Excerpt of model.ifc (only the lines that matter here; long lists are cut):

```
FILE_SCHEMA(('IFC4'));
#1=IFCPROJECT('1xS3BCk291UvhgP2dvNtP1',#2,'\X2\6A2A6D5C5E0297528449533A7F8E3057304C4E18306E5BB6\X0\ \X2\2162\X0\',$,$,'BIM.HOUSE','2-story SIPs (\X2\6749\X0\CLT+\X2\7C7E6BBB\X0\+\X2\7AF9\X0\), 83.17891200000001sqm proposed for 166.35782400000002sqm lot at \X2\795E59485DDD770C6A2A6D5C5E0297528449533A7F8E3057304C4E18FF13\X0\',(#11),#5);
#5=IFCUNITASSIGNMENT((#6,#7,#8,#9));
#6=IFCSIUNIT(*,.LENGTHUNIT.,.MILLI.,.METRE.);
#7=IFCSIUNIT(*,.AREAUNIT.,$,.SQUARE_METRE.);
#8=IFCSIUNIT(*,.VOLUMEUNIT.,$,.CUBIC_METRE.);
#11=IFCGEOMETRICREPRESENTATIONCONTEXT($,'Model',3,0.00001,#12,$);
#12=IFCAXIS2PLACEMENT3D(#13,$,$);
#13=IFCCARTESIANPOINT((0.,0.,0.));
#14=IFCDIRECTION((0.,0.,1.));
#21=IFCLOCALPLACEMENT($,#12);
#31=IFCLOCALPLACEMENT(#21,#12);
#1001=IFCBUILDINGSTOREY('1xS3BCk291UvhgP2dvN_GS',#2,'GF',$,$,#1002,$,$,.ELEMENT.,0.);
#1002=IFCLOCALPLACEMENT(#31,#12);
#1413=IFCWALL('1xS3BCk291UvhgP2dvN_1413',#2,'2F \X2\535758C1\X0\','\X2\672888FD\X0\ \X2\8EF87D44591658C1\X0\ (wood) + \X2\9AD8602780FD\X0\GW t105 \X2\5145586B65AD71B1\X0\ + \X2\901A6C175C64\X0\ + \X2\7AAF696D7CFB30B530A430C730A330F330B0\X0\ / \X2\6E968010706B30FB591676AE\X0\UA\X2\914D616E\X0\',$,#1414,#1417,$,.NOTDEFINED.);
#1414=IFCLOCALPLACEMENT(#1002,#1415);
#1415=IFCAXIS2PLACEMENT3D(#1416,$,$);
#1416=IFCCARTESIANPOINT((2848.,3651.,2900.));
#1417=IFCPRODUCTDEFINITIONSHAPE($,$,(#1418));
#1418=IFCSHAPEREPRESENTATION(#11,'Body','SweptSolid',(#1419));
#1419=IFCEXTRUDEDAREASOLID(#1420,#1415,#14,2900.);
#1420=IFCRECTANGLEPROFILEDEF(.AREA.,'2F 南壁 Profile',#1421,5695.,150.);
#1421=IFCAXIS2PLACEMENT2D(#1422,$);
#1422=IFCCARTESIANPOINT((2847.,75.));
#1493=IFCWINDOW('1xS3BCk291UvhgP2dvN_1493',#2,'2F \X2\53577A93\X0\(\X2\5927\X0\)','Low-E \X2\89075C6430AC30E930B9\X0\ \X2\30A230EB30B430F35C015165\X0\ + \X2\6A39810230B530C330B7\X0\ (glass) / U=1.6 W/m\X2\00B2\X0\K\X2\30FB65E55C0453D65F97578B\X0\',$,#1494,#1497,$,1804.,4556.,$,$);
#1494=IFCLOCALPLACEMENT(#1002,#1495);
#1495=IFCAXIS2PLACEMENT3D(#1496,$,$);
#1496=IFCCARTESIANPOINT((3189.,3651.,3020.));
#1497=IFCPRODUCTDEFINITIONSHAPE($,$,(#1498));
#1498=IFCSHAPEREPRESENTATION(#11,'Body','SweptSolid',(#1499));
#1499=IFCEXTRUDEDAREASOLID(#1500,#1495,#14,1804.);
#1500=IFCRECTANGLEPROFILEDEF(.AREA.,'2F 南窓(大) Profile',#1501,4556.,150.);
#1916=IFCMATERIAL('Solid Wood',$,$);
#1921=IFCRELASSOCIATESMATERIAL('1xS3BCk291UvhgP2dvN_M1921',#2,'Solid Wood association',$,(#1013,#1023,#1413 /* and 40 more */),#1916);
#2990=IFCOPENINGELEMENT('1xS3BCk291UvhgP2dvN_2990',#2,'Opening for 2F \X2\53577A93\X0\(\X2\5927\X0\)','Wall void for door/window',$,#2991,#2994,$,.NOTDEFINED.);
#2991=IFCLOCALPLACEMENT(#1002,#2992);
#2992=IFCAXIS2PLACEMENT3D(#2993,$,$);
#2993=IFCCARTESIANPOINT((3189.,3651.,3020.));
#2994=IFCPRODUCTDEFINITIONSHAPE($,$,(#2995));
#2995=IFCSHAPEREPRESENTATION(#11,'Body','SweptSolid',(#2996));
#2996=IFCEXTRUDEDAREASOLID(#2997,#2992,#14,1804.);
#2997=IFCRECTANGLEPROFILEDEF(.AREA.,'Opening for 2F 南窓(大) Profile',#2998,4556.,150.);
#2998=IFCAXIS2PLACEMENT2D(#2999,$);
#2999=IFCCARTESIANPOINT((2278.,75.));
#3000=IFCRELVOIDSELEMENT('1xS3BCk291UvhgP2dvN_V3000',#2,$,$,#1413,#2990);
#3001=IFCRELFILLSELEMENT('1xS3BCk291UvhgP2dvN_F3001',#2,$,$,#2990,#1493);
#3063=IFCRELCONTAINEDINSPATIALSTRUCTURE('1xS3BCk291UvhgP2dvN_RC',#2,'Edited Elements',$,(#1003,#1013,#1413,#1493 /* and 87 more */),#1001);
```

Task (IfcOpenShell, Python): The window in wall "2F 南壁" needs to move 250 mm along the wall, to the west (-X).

```python
import ifcopenshell
import ifcopenshell.api.geometry
import ifcopenshell.util.placement

model = ifcopenshell.open("model.ifc")

window = model.by_guid("1xS3BCk291UvhgP2dvN_1493")
opening = window.FillsVoids[0].RelatingOpeningElement
wall = opening.VoidsElements[0].RelatingBuildingElement

wall_matrix = ifcopenshell.util.placement.get_local_placement(wall.ObjectPlacement)
shift = wall_matrix[:3, 0] * -250.0
before = ifcopenshell.util.placement.get_local_placement(window.ObjectPlacement)[:3, 3].copy()

# The window is not placed relative to its opening, so move both.
for product in (opening, window):
    matrix = ifcopenshell.util.placement.get_local_placement(product.ObjectPlacement)
    matrix[:3, 3] += shift
    ifcopenshell.api.geometry.edit_object_placement(model, product=product, matrix=matrix, is_si=False)

after = ifcopenshell.util.placement.get_local_placement(window.ObjectPlacement)[:3, 3]
print("window moved by", (after - before).round(3) + 0.0)

model.write("model_updated.ifc")
```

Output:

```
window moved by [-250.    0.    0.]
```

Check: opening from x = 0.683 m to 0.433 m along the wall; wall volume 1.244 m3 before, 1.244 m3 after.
